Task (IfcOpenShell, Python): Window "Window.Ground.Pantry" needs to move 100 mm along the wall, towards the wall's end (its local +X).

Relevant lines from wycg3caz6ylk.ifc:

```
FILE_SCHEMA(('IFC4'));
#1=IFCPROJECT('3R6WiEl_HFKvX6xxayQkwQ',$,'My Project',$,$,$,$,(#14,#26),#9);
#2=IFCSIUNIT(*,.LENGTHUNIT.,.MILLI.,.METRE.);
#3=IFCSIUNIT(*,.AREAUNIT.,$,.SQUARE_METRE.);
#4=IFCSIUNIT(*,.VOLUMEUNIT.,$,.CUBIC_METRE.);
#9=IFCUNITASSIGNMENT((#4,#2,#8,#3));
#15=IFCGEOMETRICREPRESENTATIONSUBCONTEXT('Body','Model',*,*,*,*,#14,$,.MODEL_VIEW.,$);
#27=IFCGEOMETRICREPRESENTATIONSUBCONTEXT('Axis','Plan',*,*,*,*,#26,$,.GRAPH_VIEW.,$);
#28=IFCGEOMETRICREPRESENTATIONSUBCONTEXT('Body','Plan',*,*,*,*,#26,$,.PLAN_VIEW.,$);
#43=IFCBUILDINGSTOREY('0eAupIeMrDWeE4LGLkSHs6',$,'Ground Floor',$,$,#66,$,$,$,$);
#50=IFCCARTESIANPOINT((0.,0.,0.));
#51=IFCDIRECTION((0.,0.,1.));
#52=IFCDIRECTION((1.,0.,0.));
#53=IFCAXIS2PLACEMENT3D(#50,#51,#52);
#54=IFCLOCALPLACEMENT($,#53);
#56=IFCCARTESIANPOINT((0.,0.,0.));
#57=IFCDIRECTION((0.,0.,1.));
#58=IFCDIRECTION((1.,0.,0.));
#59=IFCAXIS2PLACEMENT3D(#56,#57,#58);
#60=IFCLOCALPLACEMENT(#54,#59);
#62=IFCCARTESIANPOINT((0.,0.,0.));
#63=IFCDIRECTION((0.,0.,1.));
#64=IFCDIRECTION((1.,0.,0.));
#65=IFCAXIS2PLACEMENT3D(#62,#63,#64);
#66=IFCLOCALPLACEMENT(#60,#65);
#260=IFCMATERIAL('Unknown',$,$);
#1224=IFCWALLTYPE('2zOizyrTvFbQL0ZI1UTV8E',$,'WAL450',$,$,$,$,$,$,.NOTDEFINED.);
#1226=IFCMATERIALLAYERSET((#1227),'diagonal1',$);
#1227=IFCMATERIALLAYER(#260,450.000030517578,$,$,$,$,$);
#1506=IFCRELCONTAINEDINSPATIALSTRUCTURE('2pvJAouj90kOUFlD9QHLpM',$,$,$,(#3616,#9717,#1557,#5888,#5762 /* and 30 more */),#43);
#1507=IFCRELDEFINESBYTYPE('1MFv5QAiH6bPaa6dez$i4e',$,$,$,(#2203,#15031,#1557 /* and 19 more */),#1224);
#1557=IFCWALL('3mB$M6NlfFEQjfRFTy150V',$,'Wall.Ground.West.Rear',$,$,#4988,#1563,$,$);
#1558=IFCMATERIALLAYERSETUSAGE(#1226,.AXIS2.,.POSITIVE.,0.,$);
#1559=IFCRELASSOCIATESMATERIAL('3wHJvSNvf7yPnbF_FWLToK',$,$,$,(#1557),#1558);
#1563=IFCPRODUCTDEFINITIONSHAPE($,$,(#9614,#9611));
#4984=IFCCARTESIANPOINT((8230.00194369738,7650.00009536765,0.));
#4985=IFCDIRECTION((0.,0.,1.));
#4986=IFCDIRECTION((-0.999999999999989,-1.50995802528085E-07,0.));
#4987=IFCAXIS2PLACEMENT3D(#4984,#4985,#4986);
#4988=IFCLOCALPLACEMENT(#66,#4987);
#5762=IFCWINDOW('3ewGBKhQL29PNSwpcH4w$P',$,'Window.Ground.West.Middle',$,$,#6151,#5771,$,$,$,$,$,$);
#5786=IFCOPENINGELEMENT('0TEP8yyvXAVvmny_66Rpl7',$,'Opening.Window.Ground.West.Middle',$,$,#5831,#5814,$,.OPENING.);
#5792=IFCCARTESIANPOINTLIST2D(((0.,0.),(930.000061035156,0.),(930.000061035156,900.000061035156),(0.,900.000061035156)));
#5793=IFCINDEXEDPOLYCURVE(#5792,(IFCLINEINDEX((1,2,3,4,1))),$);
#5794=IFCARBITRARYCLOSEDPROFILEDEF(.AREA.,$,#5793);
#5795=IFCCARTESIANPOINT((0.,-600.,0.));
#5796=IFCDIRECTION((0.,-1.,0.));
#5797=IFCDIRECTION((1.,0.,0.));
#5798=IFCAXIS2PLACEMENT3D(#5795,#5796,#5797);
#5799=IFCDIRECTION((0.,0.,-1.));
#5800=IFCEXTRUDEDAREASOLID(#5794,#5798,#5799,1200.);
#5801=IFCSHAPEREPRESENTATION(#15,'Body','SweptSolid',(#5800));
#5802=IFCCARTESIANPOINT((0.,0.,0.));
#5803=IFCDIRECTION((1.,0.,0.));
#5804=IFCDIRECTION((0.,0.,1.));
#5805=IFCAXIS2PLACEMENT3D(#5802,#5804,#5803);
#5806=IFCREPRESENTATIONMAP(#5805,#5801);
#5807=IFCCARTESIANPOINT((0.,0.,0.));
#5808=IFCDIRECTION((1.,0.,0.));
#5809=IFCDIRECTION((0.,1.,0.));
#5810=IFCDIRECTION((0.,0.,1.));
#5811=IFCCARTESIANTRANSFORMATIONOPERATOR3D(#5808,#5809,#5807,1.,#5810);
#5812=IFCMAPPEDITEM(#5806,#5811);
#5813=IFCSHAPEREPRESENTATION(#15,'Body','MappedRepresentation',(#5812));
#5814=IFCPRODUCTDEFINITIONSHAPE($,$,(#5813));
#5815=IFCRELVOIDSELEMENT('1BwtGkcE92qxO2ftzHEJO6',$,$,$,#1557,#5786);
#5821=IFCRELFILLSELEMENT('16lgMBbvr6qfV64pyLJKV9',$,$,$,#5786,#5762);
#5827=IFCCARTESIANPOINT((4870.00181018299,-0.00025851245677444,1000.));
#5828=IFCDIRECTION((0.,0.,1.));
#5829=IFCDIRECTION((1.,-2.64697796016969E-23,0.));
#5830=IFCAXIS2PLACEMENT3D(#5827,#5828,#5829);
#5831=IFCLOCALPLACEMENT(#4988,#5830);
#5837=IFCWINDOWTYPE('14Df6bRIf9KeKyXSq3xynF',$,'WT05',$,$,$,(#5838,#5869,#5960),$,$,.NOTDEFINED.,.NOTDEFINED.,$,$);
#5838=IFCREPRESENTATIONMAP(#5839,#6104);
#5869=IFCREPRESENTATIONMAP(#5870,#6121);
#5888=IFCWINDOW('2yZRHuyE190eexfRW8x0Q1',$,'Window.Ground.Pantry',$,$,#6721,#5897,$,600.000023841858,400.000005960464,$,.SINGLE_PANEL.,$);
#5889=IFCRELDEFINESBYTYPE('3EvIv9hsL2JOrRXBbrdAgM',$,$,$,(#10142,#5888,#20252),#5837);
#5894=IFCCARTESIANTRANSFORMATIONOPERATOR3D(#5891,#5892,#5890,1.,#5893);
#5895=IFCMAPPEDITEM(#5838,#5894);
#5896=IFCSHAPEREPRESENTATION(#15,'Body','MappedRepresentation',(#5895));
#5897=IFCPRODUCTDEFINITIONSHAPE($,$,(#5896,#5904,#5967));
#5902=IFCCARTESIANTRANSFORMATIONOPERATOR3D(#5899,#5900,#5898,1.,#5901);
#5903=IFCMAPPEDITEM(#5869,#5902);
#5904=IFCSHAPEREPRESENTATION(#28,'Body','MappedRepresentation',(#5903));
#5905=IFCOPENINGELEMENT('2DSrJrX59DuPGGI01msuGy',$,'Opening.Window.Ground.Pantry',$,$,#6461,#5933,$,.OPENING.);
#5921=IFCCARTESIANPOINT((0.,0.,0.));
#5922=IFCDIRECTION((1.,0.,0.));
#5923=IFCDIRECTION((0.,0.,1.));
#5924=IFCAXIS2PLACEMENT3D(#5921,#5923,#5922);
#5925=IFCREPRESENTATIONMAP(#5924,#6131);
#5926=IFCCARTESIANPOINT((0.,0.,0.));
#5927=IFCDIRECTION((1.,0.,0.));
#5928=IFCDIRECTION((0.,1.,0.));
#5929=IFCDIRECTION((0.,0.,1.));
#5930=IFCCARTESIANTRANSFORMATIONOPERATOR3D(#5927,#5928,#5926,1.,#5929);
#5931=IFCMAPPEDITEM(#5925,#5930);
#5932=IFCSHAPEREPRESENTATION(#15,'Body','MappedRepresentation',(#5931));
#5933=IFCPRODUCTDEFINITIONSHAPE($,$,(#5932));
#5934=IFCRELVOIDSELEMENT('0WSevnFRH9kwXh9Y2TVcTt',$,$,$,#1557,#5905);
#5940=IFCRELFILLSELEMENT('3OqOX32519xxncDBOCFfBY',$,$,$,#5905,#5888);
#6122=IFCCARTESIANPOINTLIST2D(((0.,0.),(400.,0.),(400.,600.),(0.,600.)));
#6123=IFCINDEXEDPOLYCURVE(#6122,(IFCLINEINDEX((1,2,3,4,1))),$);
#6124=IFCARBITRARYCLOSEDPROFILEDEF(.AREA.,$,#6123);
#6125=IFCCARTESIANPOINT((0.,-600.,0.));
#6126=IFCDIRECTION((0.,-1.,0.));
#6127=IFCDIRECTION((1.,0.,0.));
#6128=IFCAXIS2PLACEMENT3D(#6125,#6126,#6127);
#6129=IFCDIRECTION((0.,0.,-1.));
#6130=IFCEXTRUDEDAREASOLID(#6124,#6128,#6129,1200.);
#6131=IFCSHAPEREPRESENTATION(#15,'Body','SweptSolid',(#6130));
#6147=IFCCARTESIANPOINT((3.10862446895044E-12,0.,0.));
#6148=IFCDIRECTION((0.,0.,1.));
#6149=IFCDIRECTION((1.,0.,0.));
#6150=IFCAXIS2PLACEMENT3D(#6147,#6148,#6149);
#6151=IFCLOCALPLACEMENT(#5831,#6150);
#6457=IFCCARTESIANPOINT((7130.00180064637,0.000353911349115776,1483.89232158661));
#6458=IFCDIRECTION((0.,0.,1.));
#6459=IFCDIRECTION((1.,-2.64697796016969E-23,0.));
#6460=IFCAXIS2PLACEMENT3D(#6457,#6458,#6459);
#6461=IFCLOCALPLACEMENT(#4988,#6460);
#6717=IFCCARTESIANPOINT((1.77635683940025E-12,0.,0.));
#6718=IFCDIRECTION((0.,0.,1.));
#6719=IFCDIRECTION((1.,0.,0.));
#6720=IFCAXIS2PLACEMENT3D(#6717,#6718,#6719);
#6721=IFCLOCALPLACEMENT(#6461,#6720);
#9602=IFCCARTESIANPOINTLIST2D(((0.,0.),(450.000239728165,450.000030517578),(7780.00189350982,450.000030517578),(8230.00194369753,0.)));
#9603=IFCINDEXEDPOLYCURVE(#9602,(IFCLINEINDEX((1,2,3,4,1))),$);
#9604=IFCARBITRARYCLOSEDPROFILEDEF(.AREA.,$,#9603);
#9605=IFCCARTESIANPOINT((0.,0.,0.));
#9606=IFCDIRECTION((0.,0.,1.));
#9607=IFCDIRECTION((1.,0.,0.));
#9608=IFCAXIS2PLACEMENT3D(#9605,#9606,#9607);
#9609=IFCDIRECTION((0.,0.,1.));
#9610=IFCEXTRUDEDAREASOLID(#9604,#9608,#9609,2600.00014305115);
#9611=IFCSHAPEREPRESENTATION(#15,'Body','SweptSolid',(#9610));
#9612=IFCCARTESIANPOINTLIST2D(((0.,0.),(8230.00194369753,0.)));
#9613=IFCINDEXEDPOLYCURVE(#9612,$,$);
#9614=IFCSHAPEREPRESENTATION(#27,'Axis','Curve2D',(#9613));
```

```python
import ifcopenshell
import ifcopenshell.api.geometry
import ifcopenshell.util.placement
import ifcopenshell.util.unit

model = ifcopenshell.open("wycg3caz6ylk.ifc")
unit_scale = ifcopenshell.util.unit.calculate_unit_scale(model)

window = model.by_guid("2yZRHuyE190eexfRW8x0Q1")
opening = window.FillsVoids[0].RelatingOpeningElement
wall = opening.VoidsElements[0].RelatingBuildingElement

wall_matrix = ifcopenshell.util.placement.get_local_placement(wall.ObjectPlacement)
shift = wall_matrix[:3, 0] * 0.1 / unit_scale
before = ifcopenshell.util.placement.get_local_placement(window.ObjectPlacement)[:3, 3].copy()

# The window is placed relative to its opening, so it follows when the opening moves.
matrix = ifcopenshell.util.placement.get_local_placement(opening.ObjectPlacement)
matrix[:3, 3] += shift
ifcopenshell.api.geometry.edit_object_placement(
    model, product=opening, matrix=matrix, is_si=False, should_transform_children=True
)

after = ifcopenshell.util.placement.get_local_placement(window.ObjectPlacement)[:3, 3]
print("window moved by", (after - before).round(3) + 0.0)

model.write("wycg3caz6ylk-out.ifc")
```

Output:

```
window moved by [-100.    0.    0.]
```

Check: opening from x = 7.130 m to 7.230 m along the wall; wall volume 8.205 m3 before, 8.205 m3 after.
